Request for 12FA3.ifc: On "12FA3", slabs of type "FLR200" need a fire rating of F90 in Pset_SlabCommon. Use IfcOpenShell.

First a look at what the model holds.

```python
import ifcopenshell
import ifcopenshell.util.element

model = ifcopenshell.open("12FA3.ifc")
print(model.schema)
storey = next(s for s in model.by_type("IfcBuildingStorey") if s.Name == "12FA3")
slabs = [e for e in ifcopenshell.util.element.get_decomposition(storey) if e.is_a("IfcSlab")]
seen = {}
for e in slabs:
    element_type = ifcopenshell.util.element.get_type(e)
    key = (element_type.Name if element_type != e and element_type else None, ifcopenshell.util.element.get_pset(e, "Pset_SlabCommon", "FireRating"))
    seen[key] = seen.get(key, 0) + 1
for (name, value), count in sorted(seen.items(), key=str):
    print(count, "x", name, "|", value)
```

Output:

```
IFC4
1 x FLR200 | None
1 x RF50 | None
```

```python
import ifcopenshell
import ifcopenshell.api.pset
import ifcopenshell.util.element

model = ifcopenshell.open("12FA3.ifc")

storey = next(s for s in model.by_type("IfcBuildingStorey") if s.Name == "12FA3")
slabs = [e for e in ifcopenshell.util.element.get_decomposition(storey) if e.is_a("IfcSlab")]

count = 0
for e in slabs:
    element_type = ifcopenshell.util.element.get_type(e)
    if element_type in (None, e) or element_type.Name != "FLR200":
        continue
    # add_pset returns the element's existing set when there is one.
    pset = ifcopenshell.api.pset.add_pset(model, product=e, name="Pset_SlabCommon")
    ifcopenshell.api.pset.edit_pset(model, pset=pset, properties={"FireRating": "F90"})
    count += 1

print(count, "slabs updated")

model.write("12FA3-out.ifc")
```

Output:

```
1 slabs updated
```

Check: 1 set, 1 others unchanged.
